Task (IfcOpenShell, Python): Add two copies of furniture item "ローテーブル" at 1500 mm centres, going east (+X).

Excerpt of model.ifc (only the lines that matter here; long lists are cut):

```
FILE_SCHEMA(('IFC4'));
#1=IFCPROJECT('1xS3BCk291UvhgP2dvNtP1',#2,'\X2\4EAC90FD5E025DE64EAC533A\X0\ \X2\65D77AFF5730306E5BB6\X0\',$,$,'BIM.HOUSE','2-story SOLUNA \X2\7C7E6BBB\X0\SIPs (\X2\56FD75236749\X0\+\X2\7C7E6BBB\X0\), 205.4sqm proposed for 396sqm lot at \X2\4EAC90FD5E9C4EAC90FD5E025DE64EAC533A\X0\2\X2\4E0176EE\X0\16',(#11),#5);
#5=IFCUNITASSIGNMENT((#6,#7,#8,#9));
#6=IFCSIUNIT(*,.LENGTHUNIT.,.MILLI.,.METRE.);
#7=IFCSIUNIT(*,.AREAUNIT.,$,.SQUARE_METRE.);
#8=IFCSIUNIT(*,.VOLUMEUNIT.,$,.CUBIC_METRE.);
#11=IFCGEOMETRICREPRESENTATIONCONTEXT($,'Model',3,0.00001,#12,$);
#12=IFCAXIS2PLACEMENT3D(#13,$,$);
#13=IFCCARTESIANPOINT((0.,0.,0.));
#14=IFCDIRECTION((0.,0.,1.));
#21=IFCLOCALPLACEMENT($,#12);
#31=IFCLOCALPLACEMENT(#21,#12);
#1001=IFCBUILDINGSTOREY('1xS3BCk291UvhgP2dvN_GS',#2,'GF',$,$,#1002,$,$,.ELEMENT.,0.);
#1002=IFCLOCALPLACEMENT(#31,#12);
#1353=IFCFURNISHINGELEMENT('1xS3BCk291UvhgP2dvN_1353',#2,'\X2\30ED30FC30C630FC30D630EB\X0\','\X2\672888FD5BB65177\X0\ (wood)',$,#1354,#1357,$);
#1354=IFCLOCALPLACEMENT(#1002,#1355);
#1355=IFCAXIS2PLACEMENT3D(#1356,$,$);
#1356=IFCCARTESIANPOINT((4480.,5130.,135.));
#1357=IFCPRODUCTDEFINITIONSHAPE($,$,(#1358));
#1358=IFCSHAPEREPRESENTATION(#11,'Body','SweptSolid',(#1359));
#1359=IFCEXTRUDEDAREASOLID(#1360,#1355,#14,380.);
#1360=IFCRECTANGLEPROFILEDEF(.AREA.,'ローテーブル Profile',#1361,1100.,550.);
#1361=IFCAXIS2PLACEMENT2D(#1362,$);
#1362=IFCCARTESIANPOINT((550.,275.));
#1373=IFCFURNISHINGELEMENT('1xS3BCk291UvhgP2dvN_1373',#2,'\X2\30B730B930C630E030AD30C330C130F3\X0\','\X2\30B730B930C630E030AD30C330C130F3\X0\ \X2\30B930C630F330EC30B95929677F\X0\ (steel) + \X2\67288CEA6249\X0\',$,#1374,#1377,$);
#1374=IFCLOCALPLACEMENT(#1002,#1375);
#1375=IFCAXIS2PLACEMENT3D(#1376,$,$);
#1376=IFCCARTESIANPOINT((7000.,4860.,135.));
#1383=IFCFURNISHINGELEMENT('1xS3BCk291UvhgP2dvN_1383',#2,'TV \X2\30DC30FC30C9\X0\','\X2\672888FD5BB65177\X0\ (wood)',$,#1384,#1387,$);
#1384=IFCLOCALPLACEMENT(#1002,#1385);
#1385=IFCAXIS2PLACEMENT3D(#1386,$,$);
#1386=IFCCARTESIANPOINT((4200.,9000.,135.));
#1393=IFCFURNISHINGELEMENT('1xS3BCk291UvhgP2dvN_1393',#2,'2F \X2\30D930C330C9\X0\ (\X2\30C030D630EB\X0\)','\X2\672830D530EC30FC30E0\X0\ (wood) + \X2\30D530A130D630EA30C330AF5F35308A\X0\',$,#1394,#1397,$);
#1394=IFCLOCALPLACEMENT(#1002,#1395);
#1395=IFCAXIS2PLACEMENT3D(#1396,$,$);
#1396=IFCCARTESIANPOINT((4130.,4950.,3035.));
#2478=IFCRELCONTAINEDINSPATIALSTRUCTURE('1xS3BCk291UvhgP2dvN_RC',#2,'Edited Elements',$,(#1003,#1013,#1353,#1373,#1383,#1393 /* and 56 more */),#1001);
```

```python
import numpy as np
import ifcopenshell
import ifcopenshell.api.geometry
import ifcopenshell.api.root
import ifcopenshell.util.element
import ifcopenshell.util.placement

model = ifcopenshell.open("model.ifc")


def reuse_history(source, copy):
    """copy_class also copies each property set's owner history, people and application; keep the originals."""
    for rel in copy.IsDefinedBy:
        if rel.is_a("IfcRelDefinesByProperties") and (history := rel.RelatingPropertyDefinition.OwnerHistory):
            rel.RelatingPropertyDefinition.OwnerHistory = source.OwnerHistory
            ifcopenshell.util.element.remove_deep2(model, history)


source = model.by_guid("1xS3BCk291UvhgP2dvN_1353")
base = ifcopenshell.util.placement.get_local_placement(source.ObjectPlacement)
step = np.array([1.0, 0.0, 0.0]) * 1500.0

for i in range(1, 3):
    copy = ifcopenshell.api.root.copy_class(model, product=source)
    copy.Representation = ifcopenshell.util.element.copy_deep(
        model, source.Representation, exclude=["IfcGeometricRepresentationContext", "IfcRepresentationMap"]
    )
    reuse_history(source, copy)
    matrix = base.copy()
    matrix[:3, 3] += i * step
    print("added at", matrix[:3, 3].round(3) + 0.0)
    ifcopenshell.api.geometry.edit_object_placement(model, product=copy, matrix=matrix, is_si=False)

model.write("model_updated.ifc")
```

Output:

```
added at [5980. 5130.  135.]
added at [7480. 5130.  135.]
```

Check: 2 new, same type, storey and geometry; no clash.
